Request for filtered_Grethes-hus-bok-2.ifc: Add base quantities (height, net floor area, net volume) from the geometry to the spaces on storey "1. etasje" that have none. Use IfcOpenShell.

First a look at what the model holds.

```python
import ifcopenshell
import ifcopenshell.util.element
import ifcopenshell.util.unit

model = ifcopenshell.open("filtered_Grethes-hus-bok-2.ifc")
print(model.schema)
for unit_type in ("LENGTHUNIT", "AREAUNIT", "VOLUMEUNIT"):
    print(unit_type, ifcopenshell.util.unit.calculate_unit_scale(model, unit_type))
storey = next(s for s in model.by_type("IfcBuildingStorey") if s.Name == "1. etasje")
spaces = [e for e in ifcopenshell.util.element.get_decomposition(storey) if e.is_a("IfcSpace")]
for e in sorted(spaces, key=lambda e: e.id()):
    print(e.id(), e.is_a(), e.Name, list(ifcopenshell.util.element.get_psets(e, qtos_only=True)), sep=" | ")
```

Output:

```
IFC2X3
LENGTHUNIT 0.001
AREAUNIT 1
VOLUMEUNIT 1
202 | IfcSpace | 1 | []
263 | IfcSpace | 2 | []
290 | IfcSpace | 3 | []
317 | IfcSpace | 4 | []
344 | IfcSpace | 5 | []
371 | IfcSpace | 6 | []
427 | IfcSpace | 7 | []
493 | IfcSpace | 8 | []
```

```python
import ifcopenshell
import ifcopenshell.api.pset
import ifcopenshell.geom
import ifcopenshell.util.element
import ifcopenshell.util.shape
import ifcopenshell.util.unit

model = ifcopenshell.open("filtered_Grethes-hus-bok-2.ifc")
unit_scale = ifcopenshell.util.unit.calculate_unit_scale(model)
area_scale = ifcopenshell.util.unit.calculate_unit_scale(model, "AREAUNIT")
volume_scale = ifcopenshell.util.unit.calculate_unit_scale(model, "VOLUMEUNIT")
settings = ifcopenshell.geom.settings()

storey = next(s for s in model.by_type("IfcBuildingStorey") if s.Name == "1. etasje")
spaces = [e for e in ifcopenshell.util.element.get_decomposition(storey) if e.is_a("IfcSpace")]

for e in sorted(spaces, key=lambda e: e.id()):
    if ifcopenshell.util.element.get_psets(e, qtos_only=True, should_inherit=False):
        continue
    # Geometry comes back in metres, in the element's own axes.
    shape = ifcopenshell.geom.create_shape(settings, e)
    values = {
        "Height": ifcopenshell.util.shape.get_z(shape.geometry) / unit_scale,
        "NetFloorArea": ifcopenshell.util.shape.get_footprint_area(shape.geometry) / area_scale,
        "NetVolume": ifcopenshell.util.shape.get_volume(shape.geometry) / volume_scale,
    }
    qto = ifcopenshell.api.pset.add_qto(model, product=e, name="BaseQuantities")
    ifcopenshell.api.pset.edit_qto(model, qto=qto, properties=values)
    print(e.id(), {k: round(v, 3) for k, v in values.items()})

model.write("filtered_Grethes-hus-bok-2-out.ifc")
```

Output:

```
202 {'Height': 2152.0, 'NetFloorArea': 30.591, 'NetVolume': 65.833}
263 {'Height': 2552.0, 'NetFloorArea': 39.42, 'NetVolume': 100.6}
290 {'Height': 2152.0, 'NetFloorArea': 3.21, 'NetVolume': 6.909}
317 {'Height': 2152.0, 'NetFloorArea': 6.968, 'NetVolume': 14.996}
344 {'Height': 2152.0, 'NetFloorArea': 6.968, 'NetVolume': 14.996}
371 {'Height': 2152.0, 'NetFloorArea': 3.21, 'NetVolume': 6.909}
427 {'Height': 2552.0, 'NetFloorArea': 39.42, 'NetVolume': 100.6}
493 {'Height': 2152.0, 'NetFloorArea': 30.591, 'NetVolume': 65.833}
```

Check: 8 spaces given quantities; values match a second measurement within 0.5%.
